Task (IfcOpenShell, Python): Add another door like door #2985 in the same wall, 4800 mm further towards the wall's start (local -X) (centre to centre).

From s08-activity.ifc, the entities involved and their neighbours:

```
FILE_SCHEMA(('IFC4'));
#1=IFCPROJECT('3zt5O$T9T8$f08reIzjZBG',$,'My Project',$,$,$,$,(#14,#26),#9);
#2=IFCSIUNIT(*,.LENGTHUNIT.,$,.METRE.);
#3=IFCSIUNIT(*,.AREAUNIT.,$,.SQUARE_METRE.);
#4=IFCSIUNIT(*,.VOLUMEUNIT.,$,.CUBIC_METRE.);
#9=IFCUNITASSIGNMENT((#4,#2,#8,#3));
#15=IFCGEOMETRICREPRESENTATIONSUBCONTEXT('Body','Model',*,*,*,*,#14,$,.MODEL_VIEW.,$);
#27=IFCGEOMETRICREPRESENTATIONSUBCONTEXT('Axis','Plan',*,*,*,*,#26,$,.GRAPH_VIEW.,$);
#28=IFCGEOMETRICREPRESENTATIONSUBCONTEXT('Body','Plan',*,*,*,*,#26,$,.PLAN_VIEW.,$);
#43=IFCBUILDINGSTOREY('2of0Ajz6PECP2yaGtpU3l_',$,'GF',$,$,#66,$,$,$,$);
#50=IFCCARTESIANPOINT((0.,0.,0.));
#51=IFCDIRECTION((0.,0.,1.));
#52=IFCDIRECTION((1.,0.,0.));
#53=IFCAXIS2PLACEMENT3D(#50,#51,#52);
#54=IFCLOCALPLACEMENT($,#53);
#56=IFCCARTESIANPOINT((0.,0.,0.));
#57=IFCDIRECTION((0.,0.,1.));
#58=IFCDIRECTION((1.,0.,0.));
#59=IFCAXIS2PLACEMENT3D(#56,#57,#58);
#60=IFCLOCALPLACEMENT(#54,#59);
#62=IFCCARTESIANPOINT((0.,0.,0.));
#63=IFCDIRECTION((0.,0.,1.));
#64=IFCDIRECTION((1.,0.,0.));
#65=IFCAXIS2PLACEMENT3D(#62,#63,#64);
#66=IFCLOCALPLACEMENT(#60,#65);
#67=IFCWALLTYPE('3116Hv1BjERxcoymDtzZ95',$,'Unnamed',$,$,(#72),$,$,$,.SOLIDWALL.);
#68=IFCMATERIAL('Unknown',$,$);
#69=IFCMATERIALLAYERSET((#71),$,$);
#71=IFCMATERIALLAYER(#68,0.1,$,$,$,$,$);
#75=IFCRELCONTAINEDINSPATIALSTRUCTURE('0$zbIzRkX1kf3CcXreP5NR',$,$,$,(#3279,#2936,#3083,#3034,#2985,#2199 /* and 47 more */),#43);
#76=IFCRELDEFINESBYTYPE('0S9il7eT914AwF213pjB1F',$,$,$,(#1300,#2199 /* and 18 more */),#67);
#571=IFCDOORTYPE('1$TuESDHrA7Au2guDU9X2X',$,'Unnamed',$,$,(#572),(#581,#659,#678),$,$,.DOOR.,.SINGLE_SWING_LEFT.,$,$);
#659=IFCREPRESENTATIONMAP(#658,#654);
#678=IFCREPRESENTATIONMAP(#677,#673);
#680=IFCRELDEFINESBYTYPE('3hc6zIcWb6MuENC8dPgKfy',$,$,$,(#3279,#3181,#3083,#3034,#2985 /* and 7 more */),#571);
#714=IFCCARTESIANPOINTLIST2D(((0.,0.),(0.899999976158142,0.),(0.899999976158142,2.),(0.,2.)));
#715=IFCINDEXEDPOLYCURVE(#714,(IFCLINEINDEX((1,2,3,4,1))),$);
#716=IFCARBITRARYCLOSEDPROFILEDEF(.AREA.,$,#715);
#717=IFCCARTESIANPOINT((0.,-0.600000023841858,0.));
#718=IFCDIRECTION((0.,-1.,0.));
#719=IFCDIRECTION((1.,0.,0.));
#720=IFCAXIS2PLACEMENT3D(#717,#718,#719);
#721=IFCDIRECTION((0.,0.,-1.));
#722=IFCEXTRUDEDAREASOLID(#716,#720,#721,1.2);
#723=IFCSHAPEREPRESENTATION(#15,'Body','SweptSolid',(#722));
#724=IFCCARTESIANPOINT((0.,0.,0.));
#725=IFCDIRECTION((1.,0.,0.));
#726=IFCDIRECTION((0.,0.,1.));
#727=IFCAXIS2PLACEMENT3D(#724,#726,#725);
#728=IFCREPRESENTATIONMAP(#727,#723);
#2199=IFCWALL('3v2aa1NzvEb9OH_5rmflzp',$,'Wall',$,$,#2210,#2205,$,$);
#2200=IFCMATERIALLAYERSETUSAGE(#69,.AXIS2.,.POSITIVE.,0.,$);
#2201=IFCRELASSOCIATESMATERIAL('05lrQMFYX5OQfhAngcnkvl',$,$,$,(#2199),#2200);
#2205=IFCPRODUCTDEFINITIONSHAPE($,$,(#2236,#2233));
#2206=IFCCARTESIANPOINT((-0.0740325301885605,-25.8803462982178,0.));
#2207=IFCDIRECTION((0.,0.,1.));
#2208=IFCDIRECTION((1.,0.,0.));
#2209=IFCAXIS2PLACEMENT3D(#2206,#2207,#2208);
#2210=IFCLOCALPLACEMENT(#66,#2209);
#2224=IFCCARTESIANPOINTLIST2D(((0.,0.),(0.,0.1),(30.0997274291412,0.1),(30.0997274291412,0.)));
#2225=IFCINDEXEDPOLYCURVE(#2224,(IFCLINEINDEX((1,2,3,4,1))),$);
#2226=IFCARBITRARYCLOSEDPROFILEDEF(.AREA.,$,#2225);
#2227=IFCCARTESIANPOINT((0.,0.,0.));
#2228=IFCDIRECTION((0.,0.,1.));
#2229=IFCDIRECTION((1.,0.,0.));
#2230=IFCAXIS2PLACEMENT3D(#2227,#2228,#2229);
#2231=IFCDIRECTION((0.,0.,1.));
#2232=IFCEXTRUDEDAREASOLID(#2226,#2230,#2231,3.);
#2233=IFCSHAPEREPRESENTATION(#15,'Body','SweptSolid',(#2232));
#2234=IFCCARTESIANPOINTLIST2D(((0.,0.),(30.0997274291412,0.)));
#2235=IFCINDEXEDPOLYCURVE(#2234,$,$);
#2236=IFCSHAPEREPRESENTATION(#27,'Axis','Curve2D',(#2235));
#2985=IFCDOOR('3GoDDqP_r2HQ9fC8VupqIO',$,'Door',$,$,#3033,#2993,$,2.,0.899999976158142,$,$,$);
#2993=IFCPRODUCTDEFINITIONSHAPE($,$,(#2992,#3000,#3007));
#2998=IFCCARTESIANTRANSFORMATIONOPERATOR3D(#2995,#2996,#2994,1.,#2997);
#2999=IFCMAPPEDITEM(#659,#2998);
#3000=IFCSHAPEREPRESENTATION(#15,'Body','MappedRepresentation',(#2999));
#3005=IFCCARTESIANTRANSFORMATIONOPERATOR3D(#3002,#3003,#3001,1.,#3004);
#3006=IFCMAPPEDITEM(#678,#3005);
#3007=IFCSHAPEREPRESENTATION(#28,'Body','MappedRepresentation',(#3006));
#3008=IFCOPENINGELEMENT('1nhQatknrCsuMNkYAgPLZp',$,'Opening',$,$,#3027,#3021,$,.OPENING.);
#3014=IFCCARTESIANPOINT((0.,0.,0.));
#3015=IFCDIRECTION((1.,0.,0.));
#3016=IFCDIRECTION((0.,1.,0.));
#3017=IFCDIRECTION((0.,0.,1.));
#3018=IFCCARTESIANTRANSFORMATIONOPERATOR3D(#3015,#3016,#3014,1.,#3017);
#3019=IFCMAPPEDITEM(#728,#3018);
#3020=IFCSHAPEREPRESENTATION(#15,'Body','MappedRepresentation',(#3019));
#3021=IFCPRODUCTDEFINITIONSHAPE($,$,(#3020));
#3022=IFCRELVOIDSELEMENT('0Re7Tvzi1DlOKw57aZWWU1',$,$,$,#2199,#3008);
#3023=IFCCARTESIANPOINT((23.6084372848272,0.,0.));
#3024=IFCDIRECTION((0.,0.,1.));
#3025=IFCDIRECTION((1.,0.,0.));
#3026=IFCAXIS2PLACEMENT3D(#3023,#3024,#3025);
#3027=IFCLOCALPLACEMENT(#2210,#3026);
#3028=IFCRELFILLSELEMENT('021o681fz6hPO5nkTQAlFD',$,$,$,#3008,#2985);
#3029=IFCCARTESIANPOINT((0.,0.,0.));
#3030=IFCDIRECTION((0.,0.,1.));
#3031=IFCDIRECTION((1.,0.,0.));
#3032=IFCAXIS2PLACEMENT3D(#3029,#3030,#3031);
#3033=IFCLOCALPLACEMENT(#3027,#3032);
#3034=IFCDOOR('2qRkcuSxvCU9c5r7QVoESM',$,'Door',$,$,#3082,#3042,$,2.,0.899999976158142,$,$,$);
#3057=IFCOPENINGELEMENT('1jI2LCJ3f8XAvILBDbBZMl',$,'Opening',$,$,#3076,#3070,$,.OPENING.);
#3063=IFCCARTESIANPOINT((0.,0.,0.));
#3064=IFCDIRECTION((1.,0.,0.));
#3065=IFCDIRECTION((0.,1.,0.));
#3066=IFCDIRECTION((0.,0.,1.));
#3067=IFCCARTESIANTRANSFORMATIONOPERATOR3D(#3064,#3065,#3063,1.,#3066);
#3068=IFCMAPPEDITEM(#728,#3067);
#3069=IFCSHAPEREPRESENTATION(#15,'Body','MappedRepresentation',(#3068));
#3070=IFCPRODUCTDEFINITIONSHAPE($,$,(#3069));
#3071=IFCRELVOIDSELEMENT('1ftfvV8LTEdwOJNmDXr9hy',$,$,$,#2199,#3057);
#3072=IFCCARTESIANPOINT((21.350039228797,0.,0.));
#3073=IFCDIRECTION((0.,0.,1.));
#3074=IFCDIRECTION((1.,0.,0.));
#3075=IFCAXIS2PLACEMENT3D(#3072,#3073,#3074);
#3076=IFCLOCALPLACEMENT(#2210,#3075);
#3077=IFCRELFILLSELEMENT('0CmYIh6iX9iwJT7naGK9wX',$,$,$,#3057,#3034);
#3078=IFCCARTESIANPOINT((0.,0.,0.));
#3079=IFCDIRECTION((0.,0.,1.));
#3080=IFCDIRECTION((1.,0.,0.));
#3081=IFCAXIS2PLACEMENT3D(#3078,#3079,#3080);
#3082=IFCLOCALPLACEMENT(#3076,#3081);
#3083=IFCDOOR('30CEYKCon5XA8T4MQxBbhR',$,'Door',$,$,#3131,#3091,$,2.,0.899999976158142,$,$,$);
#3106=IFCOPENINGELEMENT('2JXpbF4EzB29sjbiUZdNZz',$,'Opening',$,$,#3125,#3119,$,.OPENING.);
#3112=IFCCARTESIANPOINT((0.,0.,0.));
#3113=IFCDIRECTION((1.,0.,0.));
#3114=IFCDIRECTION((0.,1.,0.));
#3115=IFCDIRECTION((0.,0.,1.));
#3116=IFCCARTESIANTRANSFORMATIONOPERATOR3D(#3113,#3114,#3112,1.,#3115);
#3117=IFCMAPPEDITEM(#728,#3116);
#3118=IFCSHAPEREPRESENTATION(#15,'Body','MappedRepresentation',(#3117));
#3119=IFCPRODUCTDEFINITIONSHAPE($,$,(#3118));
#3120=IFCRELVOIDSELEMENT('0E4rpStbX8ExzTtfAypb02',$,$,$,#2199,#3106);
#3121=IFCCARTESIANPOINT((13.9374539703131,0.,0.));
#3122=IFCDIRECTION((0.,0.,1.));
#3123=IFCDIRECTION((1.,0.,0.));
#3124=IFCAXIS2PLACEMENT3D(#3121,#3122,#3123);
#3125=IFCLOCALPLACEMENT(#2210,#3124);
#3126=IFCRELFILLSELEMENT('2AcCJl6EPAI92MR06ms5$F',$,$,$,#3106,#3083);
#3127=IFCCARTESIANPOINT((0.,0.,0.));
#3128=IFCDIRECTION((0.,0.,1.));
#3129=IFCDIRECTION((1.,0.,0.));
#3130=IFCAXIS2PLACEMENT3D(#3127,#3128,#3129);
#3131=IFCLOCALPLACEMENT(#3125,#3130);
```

```python
import ifcopenshell
import ifcopenshell.api.feature
import ifcopenshell.api.geometry
import ifcopenshell.api.root
import ifcopenshell.geom
import ifcopenshell.util.element
import ifcopenshell.util.placement
import ifcopenshell.util.shape
import ifcopenshell.util.unit

model = ifcopenshell.open("s08-activity.ifc")
unit_scale = ifcopenshell.util.unit.calculate_unit_scale(model)
settings = ifcopenshell.geom.settings()


def volume(element):
    """Net volume in cubic metres, openings subtracted."""
    shape = ifcopenshell.geom.create_shape(settings, element)
    return ifcopenshell.util.shape.get_volume(shape.geometry)


door = model.by_id(2985)
opening = door.FillsVoids[0].RelatingOpeningElement
wall = opening.VoidsElements[0].RelatingBuildingElement
before = volume(wall)
shift = ifcopenshell.util.placement.get_local_placement(wall.ObjectPlacement)[:3, 0] * -4.8 / unit_scale

# copy_class copies the void relationship, type, container and properties, but no geometry.
new_opening = ifcopenshell.api.root.copy_class(model, product=opening)
new_opening.Representation = ifcopenshell.util.element.copy_deep(
    model, opening.Representation, exclude=["IfcGeometricRepresentationContext", "IfcRepresentationMap"]
)
new_door = ifcopenshell.api.root.copy_class(model, product=door)
new_door.Representation = ifcopenshell.util.element.copy_deep(
    model, door.Representation, exclude=["IfcGeometricRepresentationContext", "IfcRepresentationMap"]
)
ifcopenshell.api.feature.add_filling(model, opening=new_opening, element=new_door)

for old, new in ((opening, new_opening), (door, new_door)):
    matrix = ifcopenshell.util.placement.get_local_placement(old.ObjectPlacement)
    matrix[:3, 3] += shift
    ifcopenshell.api.geometry.edit_object_placement(model, product=new, matrix=matrix, is_si=False)

after = volume(wall)

print(f"wall volume {before:.3f} -> {after:.3f} m3")

model.write("s08-activity_updated.ifc")
```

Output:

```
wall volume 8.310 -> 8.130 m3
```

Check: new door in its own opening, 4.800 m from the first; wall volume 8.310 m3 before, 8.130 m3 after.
